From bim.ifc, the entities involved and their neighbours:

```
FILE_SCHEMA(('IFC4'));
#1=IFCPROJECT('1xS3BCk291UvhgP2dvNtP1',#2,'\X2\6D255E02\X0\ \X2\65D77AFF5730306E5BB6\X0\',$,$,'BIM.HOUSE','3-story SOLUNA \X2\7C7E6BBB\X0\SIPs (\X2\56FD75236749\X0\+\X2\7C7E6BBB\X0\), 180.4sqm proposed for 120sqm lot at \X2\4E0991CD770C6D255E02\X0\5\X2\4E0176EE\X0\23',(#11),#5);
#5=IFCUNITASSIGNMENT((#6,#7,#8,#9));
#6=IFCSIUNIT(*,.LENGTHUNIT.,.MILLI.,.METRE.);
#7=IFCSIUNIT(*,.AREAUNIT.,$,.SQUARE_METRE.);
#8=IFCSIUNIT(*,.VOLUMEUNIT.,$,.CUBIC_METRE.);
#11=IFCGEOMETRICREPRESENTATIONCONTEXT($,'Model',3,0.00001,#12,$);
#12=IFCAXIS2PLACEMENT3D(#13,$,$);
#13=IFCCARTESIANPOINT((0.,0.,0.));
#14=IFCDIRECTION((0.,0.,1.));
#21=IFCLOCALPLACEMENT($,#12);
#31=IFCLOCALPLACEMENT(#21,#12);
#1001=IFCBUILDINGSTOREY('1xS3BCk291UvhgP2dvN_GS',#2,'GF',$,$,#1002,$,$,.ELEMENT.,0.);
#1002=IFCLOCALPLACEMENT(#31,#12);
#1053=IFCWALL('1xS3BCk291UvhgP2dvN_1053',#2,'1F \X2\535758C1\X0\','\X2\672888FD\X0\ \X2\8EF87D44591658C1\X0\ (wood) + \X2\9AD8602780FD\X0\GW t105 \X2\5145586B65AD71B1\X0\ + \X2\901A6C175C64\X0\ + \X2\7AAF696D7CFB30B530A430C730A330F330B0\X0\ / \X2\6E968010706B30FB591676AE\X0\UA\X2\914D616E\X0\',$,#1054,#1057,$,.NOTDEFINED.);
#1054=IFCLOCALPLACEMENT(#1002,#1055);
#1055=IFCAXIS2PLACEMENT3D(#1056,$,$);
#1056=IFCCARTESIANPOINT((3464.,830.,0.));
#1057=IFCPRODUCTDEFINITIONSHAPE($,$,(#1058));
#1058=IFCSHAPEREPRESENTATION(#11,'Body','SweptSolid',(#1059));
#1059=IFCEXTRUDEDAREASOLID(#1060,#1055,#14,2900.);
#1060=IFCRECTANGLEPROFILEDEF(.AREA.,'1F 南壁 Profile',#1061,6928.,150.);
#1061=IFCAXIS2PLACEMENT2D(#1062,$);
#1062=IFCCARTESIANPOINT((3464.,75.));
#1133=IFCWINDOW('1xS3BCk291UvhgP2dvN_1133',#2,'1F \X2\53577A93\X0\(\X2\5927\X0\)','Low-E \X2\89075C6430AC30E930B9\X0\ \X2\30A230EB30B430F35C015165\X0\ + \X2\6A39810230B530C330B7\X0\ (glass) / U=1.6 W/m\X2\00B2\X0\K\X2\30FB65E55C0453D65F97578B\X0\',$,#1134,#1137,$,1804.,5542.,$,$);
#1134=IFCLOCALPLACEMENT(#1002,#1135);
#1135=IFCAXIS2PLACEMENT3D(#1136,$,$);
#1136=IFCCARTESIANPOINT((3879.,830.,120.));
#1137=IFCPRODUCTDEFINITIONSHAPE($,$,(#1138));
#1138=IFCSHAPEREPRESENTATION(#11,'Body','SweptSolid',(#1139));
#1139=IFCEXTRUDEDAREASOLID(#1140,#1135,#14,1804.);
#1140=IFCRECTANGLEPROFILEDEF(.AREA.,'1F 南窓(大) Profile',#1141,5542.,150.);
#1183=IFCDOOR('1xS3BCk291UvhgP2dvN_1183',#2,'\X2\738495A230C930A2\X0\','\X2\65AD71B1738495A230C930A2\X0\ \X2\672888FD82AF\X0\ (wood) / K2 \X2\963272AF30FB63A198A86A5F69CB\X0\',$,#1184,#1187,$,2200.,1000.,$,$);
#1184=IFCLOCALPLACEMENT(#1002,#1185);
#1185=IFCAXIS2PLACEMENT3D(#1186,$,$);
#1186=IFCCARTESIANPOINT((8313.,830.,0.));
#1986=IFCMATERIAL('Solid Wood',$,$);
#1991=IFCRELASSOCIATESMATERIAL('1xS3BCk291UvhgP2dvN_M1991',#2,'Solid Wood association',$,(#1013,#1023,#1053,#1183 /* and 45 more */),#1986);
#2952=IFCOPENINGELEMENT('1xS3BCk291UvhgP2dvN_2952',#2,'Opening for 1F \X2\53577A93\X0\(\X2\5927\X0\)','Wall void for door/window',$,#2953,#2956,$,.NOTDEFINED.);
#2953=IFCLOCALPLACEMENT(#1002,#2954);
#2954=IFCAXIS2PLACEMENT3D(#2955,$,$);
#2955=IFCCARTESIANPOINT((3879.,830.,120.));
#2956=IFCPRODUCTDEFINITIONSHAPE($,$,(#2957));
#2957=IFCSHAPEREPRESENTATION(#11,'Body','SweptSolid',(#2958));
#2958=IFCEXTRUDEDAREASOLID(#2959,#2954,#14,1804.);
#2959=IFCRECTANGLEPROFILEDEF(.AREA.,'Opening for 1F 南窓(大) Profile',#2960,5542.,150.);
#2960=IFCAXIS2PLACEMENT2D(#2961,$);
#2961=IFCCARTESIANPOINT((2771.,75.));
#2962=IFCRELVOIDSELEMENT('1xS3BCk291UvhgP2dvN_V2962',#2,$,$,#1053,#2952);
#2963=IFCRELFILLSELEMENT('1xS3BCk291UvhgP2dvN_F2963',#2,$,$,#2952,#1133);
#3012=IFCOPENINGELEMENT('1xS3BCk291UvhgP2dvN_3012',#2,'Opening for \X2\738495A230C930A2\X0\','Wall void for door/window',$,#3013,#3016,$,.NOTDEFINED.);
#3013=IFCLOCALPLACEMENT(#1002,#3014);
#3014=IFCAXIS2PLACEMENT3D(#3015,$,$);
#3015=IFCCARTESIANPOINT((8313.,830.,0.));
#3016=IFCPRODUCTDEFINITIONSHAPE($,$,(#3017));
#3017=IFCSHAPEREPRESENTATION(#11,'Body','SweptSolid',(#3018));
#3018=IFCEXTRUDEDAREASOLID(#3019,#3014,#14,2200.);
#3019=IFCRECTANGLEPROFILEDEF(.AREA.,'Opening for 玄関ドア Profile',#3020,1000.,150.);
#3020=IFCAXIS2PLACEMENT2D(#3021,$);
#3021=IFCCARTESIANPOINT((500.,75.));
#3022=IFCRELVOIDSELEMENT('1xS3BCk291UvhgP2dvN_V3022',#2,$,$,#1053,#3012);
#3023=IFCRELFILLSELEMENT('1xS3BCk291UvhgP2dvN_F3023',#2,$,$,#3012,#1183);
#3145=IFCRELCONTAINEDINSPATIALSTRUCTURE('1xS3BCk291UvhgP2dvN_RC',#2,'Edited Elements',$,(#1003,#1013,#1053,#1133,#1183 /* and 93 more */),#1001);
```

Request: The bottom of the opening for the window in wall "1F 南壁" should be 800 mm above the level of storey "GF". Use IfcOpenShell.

```python
import numpy as np
import ifcopenshell
import ifcopenshell.api.geometry
import ifcopenshell.geom
import ifcopenshell.util.element
import ifcopenshell.util.placement
import ifcopenshell.util.shape
import ifcopenshell.util.unit

model = ifcopenshell.open("bim.ifc")
unit_scale = ifcopenshell.util.unit.calculate_unit_scale(model)

window = model.by_guid("1xS3BCk291UvhgP2dvN_1133")
opening = window.FillsVoids[0].RelatingOpeningElement
storey = ifcopenshell.util.element.get_container(window, ifc_class="IfcBuildingStorey")
level = ifcopenshell.util.placement.get_local_placement(storey.ObjectPlacement)[2, 3]

# The opening's origin need not be at the sill, so measure its lowest point.
shape = ifcopenshell.geom.create_shape(ifcopenshell.geom.settings(), opening)
bottom = ifcopenshell.util.shape.get_shape_bottom_elevation(shape, shape.geometry) / unit_scale
dz = level + 800.0 - bottom

shift = np.array([0.0, 0.0, dz])
# The window is not placed relative to its opening, so move both.
for product in (opening, window):
    matrix = ifcopenshell.util.placement.get_local_placement(product.ObjectPlacement)
    matrix[:3, 3] += shift
    ifcopenshell.api.geometry.edit_object_placement(model, product=product, matrix=matrix, is_si=False)

print(f"moved by {dz * unit_scale:+.3f} m")

model.write("bim_rev.ifc")
```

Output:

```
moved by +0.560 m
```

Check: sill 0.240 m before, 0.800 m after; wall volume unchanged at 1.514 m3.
